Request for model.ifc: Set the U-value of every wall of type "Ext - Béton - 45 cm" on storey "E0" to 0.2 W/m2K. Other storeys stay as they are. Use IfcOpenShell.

First a look at what the model holds.

```python
import ifcopenshell
import ifcopenshell.util.element

model = ifcopenshell.open("model.ifc")
print(model.schema)
storey = next(s for s in model.by_type("IfcBuildingStorey") if s.Name == "E0")
walls = [e for e in ifcopenshell.util.element.get_decomposition(storey) if e.is_a("IfcWall")]
seen = {}
for e in walls:
    element_type = ifcopenshell.util.element.get_type(e)
    key = (element_type.Name if element_type != e and element_type else None, ifcopenshell.util.element.get_pset(e, "Pset_WallCommon", "ThermalTransmittance"))
    seen[key] = seen.get(key, 0) + 1
for (name, value), count in sorted(seen.items(), key=str):
    print(count, "x", name, "|", value)
```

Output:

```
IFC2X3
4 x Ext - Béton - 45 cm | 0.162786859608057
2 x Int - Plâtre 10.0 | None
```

```python
import ifcopenshell
import ifcopenshell.api.pset
import ifcopenshell.util.element

model = ifcopenshell.open("model.ifc")

storey = next(s for s in model.by_type("IfcBuildingStorey") if s.Name == "E0")
walls = [e for e in ifcopenshell.util.element.get_decomposition(storey) if e.is_a("IfcWall")]

count = 0
for e in walls:
    element_type = ifcopenshell.util.element.get_type(e)
    if element_type in (None, e) or element_type.Name != "Ext - Béton - 45 cm":
        continue
    # add_pset returns the element's existing set when there is one.
    pset = ifcopenshell.api.pset.add_pset(model, product=e, name="Pset_WallCommon")
    ifcopenshell.api.pset.edit_pset(model, pset=pset, properties={"ThermalTransmittance": 0.2})
    count += 1

print(count, "walls updated")

model.write("model_updated.ifc")
```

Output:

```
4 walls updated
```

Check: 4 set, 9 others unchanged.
